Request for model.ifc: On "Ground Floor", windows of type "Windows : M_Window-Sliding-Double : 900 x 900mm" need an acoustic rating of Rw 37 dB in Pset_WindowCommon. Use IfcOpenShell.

First a look at what the model holds.

```python
import ifcopenshell
import ifcopenshell.util.element

model = ifcopenshell.open("model.ifc")
print(model.schema)
storey = next(s for s in model.by_type("IfcBuildingStorey") if s.Name == "Ground Floor")
windows = [e for e in ifcopenshell.util.element.get_decomposition(storey) if e.is_a("IfcWindow")]
seen = {}
for e in windows:
    element_type = ifcopenshell.util.element.get_type(e)
    key = (element_type.Name if element_type != e and element_type else None, ifcopenshell.util.element.get_pset(e, "Pset_WindowCommon", "AcousticRating"))
    seen[key] = seen.get(key, 0) + 1
for (name, value), count in sorted(seen.items(), key=str):
    print(count, "x", name, "|", value)
```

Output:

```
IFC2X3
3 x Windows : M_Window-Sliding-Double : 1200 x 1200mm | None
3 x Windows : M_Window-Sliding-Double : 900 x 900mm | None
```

```python
import ifcopenshell
import ifcopenshell.api.pset
import ifcopenshell.util.element

model = ifcopenshell.open("model.ifc")

storey = next(s for s in model.by_type("IfcBuildingStorey") if s.Name == "Ground Floor")
windows = [e for e in ifcopenshell.util.element.get_decomposition(storey) if e.is_a("IfcWindow")]

count = 0
for e in windows:
    element_type = ifcopenshell.util.element.get_type(e)
    if element_type in (None, e) or element_type.Name != "Windows : M_Window-Sliding-Double : 900 x 900mm":
        continue
    # add_pset returns the element's existing set when there is one.
    pset = ifcopenshell.api.pset.add_pset(model, product=e, name="Pset_WindowCommon")
    ifcopenshell.api.pset.edit_pset(model, pset=pset, properties={"AcousticRating": "Rw 37 dB"})
    count += 1

print(count, "windows updated")

model.write("model_rev.ifc")
```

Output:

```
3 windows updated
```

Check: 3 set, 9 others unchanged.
